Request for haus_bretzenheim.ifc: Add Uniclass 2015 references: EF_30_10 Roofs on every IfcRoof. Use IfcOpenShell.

First a look at what the model holds.

```python
import ifcopenshell

model = ifcopenshell.open("haus_bretzenheim.ifc")
print(model.schema)
print("classifications:", [c.Name for c in model.by_type("IfcClassification")])
for ifc_class in ("IfcDoor", "IfcRoof", "IfcStair", "IfcWall", "IfcWindow"):
    print(ifc_class, len(model.by_type(ifc_class)))
```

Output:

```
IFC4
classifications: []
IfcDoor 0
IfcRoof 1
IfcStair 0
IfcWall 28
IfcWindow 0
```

```python
import ifcopenshell
import ifcopenshell.api.classification

model = ifcopenshell.open("haus_bretzenheim.ifc")

system = ifcopenshell.api.classification.add_classification(model, classification="Uniclass 2015")

codes = {
    "IfcRoof": ("EF_30_10", "Roofs"),
}
for ifc_class, (code, name) in codes.items():
    products = model.by_type(ifc_class)
    ifcopenshell.api.classification.add_reference(
        model, products=products, classification=system, identification=code, name=name
    )
    print(code, len(products))

model.write("haus_bretzenheim-out.ifc")
```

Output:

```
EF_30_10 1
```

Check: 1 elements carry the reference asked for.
